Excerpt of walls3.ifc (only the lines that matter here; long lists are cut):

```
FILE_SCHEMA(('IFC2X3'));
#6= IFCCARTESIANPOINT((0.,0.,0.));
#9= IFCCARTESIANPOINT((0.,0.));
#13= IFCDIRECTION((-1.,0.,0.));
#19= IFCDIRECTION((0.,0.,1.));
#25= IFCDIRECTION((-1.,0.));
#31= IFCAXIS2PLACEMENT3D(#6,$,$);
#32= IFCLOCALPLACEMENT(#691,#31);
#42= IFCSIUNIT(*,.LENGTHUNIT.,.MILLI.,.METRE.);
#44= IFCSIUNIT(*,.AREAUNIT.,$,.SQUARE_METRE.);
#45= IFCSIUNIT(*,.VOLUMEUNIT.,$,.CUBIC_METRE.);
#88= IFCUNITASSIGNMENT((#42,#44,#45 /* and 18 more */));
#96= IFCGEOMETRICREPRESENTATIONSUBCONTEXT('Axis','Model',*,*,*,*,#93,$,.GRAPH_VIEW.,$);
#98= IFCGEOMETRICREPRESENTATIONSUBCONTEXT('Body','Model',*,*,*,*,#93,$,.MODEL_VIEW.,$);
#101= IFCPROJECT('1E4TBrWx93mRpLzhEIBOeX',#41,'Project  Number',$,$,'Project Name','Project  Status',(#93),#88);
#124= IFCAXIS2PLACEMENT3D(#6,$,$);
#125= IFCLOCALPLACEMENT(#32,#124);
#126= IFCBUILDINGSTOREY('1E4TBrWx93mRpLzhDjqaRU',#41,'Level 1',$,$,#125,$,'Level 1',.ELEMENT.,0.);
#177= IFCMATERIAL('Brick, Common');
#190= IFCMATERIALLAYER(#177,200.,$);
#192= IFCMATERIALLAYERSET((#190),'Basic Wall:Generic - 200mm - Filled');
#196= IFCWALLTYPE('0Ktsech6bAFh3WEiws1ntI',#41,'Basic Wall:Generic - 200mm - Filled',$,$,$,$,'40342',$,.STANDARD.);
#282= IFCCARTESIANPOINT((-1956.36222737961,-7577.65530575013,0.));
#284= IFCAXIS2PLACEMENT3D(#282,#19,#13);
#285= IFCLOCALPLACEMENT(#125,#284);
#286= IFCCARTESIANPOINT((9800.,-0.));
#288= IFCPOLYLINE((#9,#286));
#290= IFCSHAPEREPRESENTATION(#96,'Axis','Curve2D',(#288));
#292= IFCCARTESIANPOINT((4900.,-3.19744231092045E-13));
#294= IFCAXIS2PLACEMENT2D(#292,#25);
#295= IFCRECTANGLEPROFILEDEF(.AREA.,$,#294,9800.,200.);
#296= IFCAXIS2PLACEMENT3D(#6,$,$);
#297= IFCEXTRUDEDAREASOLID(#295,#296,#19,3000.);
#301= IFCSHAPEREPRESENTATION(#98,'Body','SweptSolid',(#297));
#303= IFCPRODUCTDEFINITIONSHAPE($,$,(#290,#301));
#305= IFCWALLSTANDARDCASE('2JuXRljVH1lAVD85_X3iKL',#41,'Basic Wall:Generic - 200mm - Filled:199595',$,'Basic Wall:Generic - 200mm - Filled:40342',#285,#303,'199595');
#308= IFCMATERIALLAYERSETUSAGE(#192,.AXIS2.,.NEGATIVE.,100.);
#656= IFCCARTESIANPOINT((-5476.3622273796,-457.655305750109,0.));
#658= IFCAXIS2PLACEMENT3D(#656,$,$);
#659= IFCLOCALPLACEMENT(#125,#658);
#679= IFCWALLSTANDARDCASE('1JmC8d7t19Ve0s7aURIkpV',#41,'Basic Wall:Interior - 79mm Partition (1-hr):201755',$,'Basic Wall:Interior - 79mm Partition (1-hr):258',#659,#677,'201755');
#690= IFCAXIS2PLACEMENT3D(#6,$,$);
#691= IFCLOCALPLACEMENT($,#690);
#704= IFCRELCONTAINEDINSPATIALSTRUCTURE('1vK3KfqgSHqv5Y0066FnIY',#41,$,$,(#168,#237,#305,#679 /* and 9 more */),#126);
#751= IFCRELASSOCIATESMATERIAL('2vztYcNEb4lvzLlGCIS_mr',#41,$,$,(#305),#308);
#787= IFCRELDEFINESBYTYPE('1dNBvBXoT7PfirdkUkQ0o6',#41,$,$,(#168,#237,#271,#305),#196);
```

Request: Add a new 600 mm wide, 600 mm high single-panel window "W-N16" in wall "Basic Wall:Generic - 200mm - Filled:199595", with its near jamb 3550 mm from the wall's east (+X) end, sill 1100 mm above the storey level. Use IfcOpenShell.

```python
import numpy as np
import ifcopenshell
import ifcopenshell.api.feature
import ifcopenshell.api.geometry
import ifcopenshell.api.root
import ifcopenshell.api.spatial
import ifcopenshell.api.type
import ifcopenshell.geom
import ifcopenshell.util.element
import ifcopenshell.util.placement
import ifcopenshell.util.representation
import ifcopenshell.util.shape
import ifcopenshell.util.unit

model = ifcopenshell.open("walls3.ifc")
unit_scale = ifcopenshell.util.unit.calculate_unit_scale(model)
settings = ifcopenshell.geom.settings()


def volume(element):
    """Net volume in cubic metres, openings subtracted."""
    shape = ifcopenshell.geom.create_shape(settings, element)
    return ifcopenshell.util.shape.get_volume(shape.geometry)


wall = model.by_guid("2JuXRljVH1lAVD85_X3iKL")
storey = ifcopenshell.util.element.get_container(wall, ifc_class="IfcBuildingStorey")
context = ifcopenshell.util.representation.get_context(model, "Model", "Body", "MODEL_VIEW")
before = volume(wall)

width, height, from_end, sill = 0.6, 0.6, 3.55, 1.1  # metres

# The wall runs along its own X axis, and the end named is its -X end.
wall_shape = ifcopenshell.geom.create_shape(settings, wall)
x, y, z = ifcopenshell.util.shape.get_vertices(wall_shape.geometry).T
start = x.min() + from_end
face, thickness = float(y.min()), float(y.max() - y.min())
wall_matrix = ifcopenshell.util.placement.get_local_placement(wall.ObjectPlacement)
level = ifcopenshell.util.placement.get_local_placement(storey.ObjectPlacement)[2, 3]


def in_wall(x, y):
    """Placement at x, y metres in the wall's axes, at sill height."""
    matrix = wall_matrix.copy()
    matrix[:, 3] = wall_matrix @ np.array([x / unit_scale, y / unit_scale, 0.0, 1.0])
    matrix[2, 3] = level + sill / unit_scale
    return matrix


# Opening: a box that overshoots both wall faces by 50 mm.
opening = ifcopenshell.api.root.create_entity(model, ifc_class="IfcOpeningElement")
box = ifcopenshell.api.geometry.add_wall_representation(
    model, context=context, length=width, height=height, thickness=thickness + 0.1
)
ifcopenshell.api.geometry.assign_representation(model, product=opening, representation=box)
ifcopenshell.api.geometry.edit_object_placement(model, product=opening, matrix=in_wall(start, face - 0.05), is_si=False)
ifcopenshell.api.feature.add_feature(model, feature=opening, element=wall)

window = ifcopenshell.api.root.create_entity(model, ifc_class="IfcWindow", name="W-N16")
window.OverallWidth, window.OverallHeight = width / unit_scale, height / unit_scale
body = ifcopenshell.api.geometry.add_window_representation(
    model,
    context=context,
    overall_width=window.OverallWidth,
    overall_height=window.OverallHeight,
    partition_type="SINGLE_PANEL",
)
ifcopenshell.api.geometry.assign_representation(model, product=window, representation=body)
ifcopenshell.api.spatial.assign_container(model, products=[window], relating_structure=storey)
fills = ifcopenshell.api.feature.add_filling(model, opening=opening, element=window)
fills.OwnerHistory = window.OwnerHistory  # required in IFC2X3

# IFC2X3 keeps the operation on the window style.
style = ifcopenshell.api.root.create_entity(model, ifc_class="IfcWindowStyle", name="W-N16")
style.OperationType, style.ConstructionType = "SINGLE_PANEL", "NOTDEFINED"
style.ParameterTakesPrecedence = style.Sizeable = False
ifcopenshell.api.type.assign_type(model, related_objects=[window], relating_type=style)

# Centre the window in the wall's thickness.
ifcopenshell.api.geometry.edit_object_placement(model, product=window, matrix=in_wall(start, face), is_si=False)
window_shape = ifcopenshell.geom.create_shape(settings, window)
depth = ifcopenshell.util.shape.get_vertices(window_shape.geometry)[:, 1]
offset = face + thickness / 2 - (depth.min() + depth.max()) / 2
ifcopenshell.api.geometry.edit_object_placement(model, product=window, matrix=in_wall(start, offset), is_si=False)

after = volume(wall)

print(f"wall volume {before:.3f} -> {after:.3f} m3")

model.write("walls3_updated.ifc")
```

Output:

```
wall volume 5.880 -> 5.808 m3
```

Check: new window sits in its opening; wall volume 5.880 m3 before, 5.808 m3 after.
